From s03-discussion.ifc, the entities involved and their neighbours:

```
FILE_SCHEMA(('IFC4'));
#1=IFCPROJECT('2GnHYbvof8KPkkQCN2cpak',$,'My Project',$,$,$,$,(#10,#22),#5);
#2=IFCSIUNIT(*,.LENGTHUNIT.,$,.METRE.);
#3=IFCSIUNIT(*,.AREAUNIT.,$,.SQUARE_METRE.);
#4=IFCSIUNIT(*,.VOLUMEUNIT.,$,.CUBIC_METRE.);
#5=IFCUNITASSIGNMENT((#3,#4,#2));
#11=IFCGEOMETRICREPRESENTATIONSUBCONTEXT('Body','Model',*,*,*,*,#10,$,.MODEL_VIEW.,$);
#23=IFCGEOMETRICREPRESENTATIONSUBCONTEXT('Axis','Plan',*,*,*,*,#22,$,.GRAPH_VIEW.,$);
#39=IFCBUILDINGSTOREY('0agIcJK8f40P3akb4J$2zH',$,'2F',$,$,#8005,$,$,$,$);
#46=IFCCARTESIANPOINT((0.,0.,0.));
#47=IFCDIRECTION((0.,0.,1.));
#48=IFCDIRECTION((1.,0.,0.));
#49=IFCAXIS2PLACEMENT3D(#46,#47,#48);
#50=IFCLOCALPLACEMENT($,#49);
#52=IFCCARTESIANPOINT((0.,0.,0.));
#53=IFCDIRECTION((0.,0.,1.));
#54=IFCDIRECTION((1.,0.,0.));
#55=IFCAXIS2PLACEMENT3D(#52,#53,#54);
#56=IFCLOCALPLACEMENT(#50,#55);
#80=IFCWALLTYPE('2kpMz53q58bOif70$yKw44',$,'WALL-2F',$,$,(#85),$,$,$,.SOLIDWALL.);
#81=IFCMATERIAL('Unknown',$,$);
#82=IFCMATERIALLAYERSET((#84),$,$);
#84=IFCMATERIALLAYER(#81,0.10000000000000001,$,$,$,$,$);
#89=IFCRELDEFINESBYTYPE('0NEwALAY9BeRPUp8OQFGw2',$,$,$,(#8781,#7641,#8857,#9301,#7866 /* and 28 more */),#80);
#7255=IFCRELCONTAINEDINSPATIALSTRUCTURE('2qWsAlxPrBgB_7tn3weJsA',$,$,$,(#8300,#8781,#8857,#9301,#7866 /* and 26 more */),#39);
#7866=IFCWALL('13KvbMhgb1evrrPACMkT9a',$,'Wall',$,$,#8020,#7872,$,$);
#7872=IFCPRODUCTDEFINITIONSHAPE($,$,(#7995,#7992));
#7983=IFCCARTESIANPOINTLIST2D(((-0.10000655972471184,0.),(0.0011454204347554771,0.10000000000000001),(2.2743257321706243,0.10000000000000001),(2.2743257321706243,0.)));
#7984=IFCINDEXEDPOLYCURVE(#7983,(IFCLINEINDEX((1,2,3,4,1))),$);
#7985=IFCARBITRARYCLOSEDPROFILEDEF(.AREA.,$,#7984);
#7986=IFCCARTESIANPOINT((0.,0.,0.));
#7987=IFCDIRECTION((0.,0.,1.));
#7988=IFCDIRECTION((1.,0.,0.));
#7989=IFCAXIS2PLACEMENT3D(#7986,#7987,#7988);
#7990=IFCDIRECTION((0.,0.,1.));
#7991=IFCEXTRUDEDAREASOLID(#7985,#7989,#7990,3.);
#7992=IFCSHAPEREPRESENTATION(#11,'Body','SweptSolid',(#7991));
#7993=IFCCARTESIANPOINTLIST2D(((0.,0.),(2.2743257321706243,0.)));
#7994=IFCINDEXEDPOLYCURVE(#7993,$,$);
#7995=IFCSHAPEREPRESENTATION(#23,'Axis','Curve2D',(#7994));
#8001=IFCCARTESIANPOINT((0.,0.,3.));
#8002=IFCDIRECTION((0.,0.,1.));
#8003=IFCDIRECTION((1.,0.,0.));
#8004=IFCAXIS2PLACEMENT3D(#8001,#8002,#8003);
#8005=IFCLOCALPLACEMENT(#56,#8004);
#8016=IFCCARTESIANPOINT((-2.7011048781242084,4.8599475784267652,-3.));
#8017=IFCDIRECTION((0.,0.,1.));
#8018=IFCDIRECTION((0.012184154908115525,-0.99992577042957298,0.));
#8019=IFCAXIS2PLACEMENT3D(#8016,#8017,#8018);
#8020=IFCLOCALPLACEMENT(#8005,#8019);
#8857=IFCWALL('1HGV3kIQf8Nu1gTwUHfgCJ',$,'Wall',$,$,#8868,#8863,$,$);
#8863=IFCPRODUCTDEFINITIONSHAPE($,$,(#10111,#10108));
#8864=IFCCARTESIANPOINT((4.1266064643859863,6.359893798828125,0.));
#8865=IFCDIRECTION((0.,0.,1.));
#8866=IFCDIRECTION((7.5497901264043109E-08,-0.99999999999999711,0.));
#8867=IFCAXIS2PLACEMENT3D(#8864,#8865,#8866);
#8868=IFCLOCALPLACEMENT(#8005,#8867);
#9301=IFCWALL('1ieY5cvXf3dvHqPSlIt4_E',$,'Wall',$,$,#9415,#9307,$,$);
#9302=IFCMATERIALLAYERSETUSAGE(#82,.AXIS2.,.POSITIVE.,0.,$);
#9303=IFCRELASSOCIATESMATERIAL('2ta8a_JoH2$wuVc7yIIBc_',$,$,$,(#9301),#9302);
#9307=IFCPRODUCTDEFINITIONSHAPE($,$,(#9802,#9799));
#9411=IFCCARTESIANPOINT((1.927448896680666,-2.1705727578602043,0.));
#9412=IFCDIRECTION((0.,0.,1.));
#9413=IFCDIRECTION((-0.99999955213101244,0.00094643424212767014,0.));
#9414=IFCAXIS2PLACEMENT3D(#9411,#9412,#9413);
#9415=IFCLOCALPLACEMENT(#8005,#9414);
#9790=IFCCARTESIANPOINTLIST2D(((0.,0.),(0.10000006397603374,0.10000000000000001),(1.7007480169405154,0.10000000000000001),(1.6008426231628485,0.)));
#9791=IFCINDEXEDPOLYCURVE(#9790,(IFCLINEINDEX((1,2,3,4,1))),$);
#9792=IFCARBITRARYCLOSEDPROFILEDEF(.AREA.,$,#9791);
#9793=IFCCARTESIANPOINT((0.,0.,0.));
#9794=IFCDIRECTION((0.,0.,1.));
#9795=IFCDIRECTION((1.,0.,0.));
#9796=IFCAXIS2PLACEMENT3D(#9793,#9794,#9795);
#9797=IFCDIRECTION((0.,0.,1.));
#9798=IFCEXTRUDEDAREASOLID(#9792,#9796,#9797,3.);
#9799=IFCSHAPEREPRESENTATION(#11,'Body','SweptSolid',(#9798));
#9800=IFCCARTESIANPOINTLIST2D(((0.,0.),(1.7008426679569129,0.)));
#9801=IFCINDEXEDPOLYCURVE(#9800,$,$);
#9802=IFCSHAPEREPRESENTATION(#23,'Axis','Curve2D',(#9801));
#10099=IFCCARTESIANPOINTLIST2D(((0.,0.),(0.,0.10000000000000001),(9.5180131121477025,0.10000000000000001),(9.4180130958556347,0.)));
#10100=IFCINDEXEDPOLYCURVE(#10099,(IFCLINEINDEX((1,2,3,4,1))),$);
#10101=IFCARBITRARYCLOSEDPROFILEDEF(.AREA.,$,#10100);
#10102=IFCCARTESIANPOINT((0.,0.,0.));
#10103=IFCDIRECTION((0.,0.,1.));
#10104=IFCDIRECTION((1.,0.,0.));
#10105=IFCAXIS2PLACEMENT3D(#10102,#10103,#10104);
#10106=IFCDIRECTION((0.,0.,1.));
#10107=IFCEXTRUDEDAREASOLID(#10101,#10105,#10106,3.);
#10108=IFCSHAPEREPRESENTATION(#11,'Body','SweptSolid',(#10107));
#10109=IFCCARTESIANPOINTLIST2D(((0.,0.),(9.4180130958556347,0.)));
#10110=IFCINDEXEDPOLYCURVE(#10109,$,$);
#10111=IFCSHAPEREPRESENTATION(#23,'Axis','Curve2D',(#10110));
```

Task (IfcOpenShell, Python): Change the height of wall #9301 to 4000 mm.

```python
import ifcopenshell
import ifcopenshell.geom
import ifcopenshell.util.representation
import ifcopenshell.util.shape

model = ifcopenshell.open("s03-discussion.ifc")
settings = ifcopenshell.geom.settings()


def volume(element):
    """Net volume in cubic metres, openings subtracted."""
    shape = ifcopenshell.geom.create_shape(settings, element)
    return ifcopenshell.util.shape.get_volume(shape.geometry)


wall = model.by_id(9301)
before = volume(wall)

body = ifcopenshell.util.representation.get_representation(wall, "Model", "Body")
solid = body.Items[0]
old_height = solid.Depth
solid.Depth = 4.0
after = volume(wall)

print(f"height {old_height:g} -> {solid.Depth:g}, volume {before:.3f} -> {after:.3f} m3")

model.write("s03-discussion_edited.ifc")
```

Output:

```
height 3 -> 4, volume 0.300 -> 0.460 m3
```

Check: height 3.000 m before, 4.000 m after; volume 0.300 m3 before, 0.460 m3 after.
